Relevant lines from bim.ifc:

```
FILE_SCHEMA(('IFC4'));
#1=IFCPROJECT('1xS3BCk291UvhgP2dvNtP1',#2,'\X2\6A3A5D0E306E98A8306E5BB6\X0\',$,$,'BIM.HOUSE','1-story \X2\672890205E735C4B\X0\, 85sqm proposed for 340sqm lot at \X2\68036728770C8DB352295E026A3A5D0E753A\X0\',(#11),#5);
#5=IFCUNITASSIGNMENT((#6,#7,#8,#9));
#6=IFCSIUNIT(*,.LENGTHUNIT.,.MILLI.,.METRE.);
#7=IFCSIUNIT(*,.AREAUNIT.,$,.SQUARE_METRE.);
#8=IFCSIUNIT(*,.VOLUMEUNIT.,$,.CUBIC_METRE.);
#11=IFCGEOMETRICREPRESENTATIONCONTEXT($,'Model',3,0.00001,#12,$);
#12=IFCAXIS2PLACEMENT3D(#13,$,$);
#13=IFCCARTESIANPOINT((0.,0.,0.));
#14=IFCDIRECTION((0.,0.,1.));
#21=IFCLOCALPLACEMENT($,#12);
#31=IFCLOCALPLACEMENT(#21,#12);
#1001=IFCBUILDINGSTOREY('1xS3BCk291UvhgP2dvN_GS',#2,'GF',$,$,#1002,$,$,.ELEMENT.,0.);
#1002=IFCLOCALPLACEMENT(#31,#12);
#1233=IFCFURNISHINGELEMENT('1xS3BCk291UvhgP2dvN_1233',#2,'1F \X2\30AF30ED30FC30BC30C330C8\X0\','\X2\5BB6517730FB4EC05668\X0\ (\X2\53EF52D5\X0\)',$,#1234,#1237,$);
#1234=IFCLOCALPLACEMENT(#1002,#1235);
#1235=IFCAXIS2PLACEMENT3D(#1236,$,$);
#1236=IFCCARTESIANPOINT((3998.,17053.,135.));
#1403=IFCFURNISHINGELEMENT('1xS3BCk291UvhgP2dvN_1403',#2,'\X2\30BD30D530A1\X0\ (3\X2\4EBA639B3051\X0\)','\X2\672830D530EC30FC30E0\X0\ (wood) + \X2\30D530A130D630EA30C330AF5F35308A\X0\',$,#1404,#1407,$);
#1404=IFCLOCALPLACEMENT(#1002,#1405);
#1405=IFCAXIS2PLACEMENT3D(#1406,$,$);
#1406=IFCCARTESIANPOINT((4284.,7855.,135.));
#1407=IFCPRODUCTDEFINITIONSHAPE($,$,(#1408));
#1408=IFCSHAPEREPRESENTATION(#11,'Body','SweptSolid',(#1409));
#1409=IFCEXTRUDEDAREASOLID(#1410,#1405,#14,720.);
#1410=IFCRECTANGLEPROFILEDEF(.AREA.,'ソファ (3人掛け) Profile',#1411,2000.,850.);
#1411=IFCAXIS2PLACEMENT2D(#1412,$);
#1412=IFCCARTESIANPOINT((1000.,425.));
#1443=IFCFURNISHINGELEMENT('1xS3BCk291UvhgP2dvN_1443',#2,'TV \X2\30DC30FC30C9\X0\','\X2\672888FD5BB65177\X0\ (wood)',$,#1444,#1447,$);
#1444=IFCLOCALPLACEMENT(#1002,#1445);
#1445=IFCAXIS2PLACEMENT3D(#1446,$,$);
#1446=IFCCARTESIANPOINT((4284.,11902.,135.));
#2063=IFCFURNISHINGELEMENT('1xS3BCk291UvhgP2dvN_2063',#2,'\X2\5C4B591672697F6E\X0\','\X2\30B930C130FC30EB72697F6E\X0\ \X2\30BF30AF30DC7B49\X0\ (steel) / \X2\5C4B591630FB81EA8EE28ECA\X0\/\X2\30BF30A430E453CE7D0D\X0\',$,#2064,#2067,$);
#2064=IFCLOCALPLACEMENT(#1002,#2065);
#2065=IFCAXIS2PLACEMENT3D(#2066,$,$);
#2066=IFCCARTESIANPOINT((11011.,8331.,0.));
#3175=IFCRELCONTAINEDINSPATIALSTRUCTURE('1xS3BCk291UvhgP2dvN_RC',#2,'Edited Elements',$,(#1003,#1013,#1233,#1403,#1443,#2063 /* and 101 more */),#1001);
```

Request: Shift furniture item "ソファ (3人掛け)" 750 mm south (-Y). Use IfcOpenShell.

```python
import ifcopenshell
import ifcopenshell.api.geometry
import ifcopenshell.util.placement

model = ifcopenshell.open("bim.ifc")

item = model.by_guid("1xS3BCk291UvhgP2dvN_1403")
matrix = ifcopenshell.util.placement.get_local_placement(item.ObjectPlacement)
matrix[1, 3] -= 750.0
ifcopenshell.api.geometry.edit_object_placement(model, product=item, matrix=matrix, is_si=False)

print(ifcopenshell.util.placement.get_local_placement(item.ObjectPlacement).round(3) + 0.0)

model.write("bim_v2.ifc")
```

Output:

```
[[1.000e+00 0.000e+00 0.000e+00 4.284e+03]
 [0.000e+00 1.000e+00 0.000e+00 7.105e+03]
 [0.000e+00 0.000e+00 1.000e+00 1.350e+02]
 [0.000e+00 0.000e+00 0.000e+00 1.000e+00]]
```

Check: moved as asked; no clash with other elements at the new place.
